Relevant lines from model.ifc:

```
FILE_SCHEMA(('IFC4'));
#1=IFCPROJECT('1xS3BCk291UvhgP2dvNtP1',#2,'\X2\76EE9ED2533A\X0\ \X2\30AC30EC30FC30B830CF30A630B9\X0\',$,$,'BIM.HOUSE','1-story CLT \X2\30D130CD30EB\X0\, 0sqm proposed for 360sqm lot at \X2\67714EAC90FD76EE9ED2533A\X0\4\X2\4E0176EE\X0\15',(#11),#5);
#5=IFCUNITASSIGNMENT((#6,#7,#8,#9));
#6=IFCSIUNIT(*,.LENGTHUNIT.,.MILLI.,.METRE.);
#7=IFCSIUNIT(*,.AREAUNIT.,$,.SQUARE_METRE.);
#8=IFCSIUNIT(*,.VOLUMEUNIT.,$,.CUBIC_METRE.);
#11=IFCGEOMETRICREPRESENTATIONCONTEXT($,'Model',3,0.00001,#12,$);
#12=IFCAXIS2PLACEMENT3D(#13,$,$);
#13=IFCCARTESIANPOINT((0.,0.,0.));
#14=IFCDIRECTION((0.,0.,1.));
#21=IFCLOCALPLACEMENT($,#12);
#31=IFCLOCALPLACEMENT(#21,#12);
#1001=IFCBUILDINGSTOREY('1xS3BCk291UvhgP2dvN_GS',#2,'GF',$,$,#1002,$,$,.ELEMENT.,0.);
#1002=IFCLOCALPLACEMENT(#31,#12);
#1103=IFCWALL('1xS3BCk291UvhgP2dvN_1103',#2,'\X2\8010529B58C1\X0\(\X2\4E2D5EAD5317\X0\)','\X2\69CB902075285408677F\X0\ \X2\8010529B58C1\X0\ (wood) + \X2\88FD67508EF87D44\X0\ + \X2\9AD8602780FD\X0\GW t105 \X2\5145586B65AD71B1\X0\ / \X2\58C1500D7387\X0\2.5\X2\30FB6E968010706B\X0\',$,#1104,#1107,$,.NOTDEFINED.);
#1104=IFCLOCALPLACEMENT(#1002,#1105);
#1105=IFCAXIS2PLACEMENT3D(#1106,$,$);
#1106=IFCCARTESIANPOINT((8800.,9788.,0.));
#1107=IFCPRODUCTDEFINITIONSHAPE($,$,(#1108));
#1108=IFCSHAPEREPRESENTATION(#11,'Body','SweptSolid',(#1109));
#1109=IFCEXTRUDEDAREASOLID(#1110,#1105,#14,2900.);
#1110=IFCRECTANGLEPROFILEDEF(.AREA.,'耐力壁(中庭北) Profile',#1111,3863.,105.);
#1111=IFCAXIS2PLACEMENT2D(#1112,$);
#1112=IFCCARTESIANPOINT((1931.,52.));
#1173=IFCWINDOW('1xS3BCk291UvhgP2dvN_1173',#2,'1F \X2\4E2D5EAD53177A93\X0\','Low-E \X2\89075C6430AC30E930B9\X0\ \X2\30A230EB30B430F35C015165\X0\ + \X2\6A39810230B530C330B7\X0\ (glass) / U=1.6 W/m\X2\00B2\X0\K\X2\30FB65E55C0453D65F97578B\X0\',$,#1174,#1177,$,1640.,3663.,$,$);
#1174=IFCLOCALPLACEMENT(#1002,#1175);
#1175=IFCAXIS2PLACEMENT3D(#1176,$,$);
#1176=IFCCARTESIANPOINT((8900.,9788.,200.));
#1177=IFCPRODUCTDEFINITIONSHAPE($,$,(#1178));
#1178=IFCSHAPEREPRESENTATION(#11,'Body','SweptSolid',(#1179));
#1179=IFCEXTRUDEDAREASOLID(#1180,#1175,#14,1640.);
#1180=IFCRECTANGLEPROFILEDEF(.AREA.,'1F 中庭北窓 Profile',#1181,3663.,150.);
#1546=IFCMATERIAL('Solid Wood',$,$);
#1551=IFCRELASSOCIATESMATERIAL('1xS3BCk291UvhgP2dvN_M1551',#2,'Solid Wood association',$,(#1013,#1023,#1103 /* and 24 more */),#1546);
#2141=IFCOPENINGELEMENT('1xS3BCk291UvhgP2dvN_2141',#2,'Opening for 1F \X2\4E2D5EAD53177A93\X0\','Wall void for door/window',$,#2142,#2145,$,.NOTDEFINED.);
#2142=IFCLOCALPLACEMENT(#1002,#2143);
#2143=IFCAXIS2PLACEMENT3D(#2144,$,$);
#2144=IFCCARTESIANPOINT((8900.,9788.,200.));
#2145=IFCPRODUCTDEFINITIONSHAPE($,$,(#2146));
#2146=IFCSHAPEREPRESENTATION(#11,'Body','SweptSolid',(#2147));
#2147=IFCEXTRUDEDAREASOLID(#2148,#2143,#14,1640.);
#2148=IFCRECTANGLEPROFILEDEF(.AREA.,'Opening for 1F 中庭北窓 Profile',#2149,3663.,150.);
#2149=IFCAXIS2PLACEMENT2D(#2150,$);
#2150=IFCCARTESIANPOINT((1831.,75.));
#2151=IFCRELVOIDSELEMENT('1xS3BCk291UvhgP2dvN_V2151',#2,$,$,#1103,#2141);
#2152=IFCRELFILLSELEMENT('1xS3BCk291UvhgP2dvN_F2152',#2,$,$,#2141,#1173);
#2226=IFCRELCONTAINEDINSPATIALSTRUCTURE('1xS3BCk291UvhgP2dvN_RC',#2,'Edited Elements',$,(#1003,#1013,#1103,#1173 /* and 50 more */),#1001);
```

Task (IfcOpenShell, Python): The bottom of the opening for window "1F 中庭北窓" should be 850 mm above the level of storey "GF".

```python
import numpy as np
import ifcopenshell
import ifcopenshell.api.geometry
import ifcopenshell.geom
import ifcopenshell.util.element
import ifcopenshell.util.placement
import ifcopenshell.util.shape
import ifcopenshell.util.unit

model = ifcopenshell.open("model.ifc")
unit_scale = ifcopenshell.util.unit.calculate_unit_scale(model)

window = model.by_guid("1xS3BCk291UvhgP2dvN_1173")
opening = window.FillsVoids[0].RelatingOpeningElement
storey = ifcopenshell.util.element.get_container(window, ifc_class="IfcBuildingStorey")
level = ifcopenshell.util.placement.get_local_placement(storey.ObjectPlacement)[2, 3]

# The opening's origin need not be at the sill, so measure its lowest point.
shape = ifcopenshell.geom.create_shape(ifcopenshell.geom.settings(), opening)
bottom = ifcopenshell.util.shape.get_shape_bottom_elevation(shape, shape.geometry) / unit_scale
dz = level + 0.85 / unit_scale - bottom

shift = np.array([0.0, 0.0, dz])
# The window is not placed relative to its opening, so move both.
for product in (opening, window):
    matrix = ifcopenshell.util.placement.get_local_placement(product.ObjectPlacement)
    matrix[:3, 3] += shift
    ifcopenshell.api.geometry.edit_object_placement(model, product=product, matrix=matrix, is_si=False)

print(f"moved by {dz * unit_scale:+.3f} m")

model.write("model_rev.ifc")
```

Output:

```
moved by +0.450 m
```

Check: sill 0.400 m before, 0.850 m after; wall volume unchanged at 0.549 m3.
